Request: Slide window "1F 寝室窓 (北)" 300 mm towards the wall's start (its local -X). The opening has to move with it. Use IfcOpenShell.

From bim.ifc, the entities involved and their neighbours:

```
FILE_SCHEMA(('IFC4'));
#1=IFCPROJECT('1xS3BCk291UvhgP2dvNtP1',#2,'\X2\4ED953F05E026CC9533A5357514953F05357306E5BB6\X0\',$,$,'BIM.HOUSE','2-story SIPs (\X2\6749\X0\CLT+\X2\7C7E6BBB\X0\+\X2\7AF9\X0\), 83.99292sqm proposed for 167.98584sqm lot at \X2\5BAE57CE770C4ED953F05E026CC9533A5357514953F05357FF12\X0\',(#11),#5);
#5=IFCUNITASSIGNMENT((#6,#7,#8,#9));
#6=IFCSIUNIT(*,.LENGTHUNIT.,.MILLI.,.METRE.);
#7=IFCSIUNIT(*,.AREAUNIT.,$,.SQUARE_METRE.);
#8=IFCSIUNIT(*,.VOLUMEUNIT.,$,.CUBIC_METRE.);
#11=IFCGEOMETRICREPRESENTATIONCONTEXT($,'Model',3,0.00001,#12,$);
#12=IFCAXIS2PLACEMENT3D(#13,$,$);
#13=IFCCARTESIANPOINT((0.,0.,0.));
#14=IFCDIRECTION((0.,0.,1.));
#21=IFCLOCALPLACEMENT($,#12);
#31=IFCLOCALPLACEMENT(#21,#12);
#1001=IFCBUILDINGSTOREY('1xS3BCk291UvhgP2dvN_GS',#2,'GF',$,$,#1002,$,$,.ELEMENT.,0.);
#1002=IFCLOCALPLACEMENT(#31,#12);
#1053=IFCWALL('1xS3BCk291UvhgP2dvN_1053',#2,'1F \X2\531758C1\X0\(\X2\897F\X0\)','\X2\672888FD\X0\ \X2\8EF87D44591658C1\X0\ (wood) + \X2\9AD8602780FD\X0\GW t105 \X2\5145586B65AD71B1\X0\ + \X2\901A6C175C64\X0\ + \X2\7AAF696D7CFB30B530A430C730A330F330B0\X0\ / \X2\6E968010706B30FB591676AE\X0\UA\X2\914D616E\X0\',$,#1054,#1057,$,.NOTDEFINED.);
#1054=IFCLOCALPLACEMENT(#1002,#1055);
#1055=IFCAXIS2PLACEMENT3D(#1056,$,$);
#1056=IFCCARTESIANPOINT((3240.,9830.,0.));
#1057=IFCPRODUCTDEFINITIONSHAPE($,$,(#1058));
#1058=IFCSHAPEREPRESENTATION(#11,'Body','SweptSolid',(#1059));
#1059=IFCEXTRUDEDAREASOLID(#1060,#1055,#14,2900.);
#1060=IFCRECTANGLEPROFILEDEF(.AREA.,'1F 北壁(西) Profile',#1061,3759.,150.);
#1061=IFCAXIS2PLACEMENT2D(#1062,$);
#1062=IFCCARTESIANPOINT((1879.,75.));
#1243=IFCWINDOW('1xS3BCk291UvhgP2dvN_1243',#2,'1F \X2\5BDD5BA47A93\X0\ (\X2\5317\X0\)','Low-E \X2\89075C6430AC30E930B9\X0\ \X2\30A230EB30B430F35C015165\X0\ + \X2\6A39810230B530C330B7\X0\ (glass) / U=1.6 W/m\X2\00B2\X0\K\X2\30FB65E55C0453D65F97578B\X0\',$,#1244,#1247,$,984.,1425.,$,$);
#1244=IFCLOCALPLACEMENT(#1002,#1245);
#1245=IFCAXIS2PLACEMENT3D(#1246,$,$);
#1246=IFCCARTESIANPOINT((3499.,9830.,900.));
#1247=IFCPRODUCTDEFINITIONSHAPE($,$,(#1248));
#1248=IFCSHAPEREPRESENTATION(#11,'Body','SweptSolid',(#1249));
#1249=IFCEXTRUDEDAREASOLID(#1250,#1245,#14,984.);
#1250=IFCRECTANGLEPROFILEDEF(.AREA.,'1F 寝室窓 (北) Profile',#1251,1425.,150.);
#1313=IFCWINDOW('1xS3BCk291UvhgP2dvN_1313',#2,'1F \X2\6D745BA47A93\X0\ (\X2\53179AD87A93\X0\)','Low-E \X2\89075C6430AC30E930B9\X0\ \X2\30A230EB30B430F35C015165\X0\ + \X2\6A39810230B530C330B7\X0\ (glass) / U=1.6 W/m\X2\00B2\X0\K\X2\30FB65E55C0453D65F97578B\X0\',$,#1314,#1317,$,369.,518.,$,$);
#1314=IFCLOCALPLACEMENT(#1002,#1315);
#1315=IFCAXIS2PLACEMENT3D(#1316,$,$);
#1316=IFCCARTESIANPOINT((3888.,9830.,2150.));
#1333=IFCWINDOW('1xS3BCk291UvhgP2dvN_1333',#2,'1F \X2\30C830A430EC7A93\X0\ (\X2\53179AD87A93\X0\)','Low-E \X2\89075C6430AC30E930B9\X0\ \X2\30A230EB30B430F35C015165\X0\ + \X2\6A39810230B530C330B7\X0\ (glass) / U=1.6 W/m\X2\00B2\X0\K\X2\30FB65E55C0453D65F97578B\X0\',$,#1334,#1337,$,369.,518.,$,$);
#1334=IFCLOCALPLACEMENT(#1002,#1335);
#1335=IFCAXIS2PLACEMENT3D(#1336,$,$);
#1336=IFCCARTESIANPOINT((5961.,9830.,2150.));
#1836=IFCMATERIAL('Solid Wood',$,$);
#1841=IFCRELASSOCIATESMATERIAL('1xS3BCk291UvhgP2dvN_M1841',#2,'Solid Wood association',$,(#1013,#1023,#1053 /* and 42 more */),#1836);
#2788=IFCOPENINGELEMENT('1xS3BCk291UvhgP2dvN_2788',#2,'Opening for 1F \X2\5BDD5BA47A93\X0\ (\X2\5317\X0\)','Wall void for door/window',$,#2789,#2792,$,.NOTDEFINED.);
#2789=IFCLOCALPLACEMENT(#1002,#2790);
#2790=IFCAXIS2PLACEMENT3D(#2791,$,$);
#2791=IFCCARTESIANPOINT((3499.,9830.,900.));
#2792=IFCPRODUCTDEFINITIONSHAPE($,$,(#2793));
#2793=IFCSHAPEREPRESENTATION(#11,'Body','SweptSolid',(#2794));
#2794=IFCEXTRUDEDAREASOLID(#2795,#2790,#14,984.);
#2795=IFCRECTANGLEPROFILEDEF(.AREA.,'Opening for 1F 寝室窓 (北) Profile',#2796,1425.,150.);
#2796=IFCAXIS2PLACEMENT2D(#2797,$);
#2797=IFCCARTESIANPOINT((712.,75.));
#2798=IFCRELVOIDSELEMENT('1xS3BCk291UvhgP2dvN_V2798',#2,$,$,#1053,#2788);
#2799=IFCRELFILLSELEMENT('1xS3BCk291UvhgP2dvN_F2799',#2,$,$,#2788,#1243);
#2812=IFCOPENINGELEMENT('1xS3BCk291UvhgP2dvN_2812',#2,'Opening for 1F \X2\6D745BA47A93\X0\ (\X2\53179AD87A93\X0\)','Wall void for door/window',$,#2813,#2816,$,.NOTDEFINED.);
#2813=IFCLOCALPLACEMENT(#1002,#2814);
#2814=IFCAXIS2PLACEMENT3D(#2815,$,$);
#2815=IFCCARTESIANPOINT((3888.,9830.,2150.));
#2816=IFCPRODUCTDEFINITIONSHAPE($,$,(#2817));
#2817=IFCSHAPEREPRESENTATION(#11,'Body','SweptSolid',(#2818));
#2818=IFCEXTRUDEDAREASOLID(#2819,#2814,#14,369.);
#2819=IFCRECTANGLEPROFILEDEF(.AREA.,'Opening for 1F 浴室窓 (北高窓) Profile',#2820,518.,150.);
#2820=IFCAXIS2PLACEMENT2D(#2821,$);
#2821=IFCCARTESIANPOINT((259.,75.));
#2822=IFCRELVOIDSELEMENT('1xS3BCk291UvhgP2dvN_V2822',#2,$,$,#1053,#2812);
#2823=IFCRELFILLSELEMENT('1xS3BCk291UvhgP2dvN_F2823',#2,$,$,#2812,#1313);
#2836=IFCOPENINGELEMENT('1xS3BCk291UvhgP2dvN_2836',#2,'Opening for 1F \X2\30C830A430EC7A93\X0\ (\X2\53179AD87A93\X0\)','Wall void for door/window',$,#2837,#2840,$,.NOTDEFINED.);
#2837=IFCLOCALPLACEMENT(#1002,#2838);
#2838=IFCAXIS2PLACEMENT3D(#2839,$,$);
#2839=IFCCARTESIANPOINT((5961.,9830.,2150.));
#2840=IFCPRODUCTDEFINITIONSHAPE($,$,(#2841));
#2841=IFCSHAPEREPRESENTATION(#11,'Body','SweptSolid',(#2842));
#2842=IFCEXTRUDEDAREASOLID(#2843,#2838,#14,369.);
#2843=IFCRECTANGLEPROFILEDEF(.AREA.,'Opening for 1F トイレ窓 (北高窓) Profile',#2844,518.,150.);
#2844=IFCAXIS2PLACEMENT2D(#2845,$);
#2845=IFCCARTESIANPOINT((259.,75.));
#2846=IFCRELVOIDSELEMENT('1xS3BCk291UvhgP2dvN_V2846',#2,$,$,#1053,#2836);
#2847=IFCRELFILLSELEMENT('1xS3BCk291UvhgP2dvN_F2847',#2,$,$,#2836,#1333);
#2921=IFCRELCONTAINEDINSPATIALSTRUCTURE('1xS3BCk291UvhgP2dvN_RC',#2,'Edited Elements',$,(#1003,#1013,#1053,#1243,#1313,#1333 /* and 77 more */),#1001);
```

```python
import ifcopenshell
import ifcopenshell.api.geometry
import ifcopenshell.util.placement

model = ifcopenshell.open("bim.ifc")

window = model.by_guid("1xS3BCk291UvhgP2dvN_1243")
opening = window.FillsVoids[0].RelatingOpeningElement
wall = opening.VoidsElements[0].RelatingBuildingElement

wall_matrix = ifcopenshell.util.placement.get_local_placement(wall.ObjectPlacement)
shift = wall_matrix[:3, 0] * -300.0
before = ifcopenshell.util.placement.get_local_placement(window.ObjectPlacement)[:3, 3].copy()

# The window is not placed relative to its opening, so move both.
for product in (opening, window):
    matrix = ifcopenshell.util.placement.get_local_placement(product.ObjectPlacement)
    matrix[:3, 3] += shift
    ifcopenshell.api.geometry.edit_object_placement(model, product=product, matrix=matrix, is_si=False)

after = ifcopenshell.util.placement.get_local_placement(window.ObjectPlacement)[:3, 3]
print("window moved by", (after - before).round(3) + 0.0)

model.write("bim_updated.ifc")
```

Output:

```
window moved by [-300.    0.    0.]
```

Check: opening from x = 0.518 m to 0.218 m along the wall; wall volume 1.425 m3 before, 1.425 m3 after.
